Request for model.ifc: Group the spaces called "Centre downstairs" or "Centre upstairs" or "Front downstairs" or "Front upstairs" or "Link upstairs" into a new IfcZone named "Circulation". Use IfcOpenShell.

First a look at what the model holds.

```python
import ifcopenshell

model = ifcopenshell.open("model.ifc")
print(model.schema)
seen = {}
for space in model.by_type("IfcSpace"):
    seen[space.Name] = seen.get(space.Name, 0) + 1
for name, count in sorted(seen.items(), key=str):
    print(count, "x", name)
print("zones:", [z.Name for z in model.by_type("IfcZone")][:20])
```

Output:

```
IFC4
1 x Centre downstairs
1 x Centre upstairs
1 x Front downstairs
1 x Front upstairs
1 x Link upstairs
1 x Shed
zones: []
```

```python
import ifcopenshell
import ifcopenshell.api.group
import ifcopenshell.api.root

model = ifcopenshell.open("model.ifc")

names = {"Centre downstairs", "Centre upstairs", "Front downstairs", "Front upstairs", "Link upstairs"}
spaces = [s for s in model.by_type("IfcSpace") if s.Name in names]

zone = ifcopenshell.api.root.create_entity(model, ifc_class="IfcZone", name="Circulation")
ifcopenshell.api.group.assign_group(model, products=spaces, group=zone)
print(len(spaces), "spaces in", zone.Name)

model.write("model_v2.ifc")
```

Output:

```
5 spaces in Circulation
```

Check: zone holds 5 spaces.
